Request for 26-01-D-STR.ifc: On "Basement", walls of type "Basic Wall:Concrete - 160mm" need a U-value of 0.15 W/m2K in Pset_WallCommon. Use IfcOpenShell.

First a look at what the model holds.

```python
import ifcopenshell
import ifcopenshell.util.element

model = ifcopenshell.open("26-01-D-STR.ifc")
print(model.schema)
storey = next(s for s in model.by_type("IfcBuildingStorey") if s.Name == "Basement")
walls = [e for e in ifcopenshell.util.element.get_decomposition(storey) if e.is_a("IfcWall")]
seen = {}
for e in walls:
    element_type = ifcopenshell.util.element.get_type(e)
    key = (element_type.Name if element_type != e and element_type else None, ifcopenshell.util.element.get_pset(e, "Pset_WallCommon", "ThermalTransmittance"))
    seen[key] = seen.get(key, 0) + 1
for (name, value), count in sorted(seen.items(), key=str):
    print(count, "x", name, "|", value)
```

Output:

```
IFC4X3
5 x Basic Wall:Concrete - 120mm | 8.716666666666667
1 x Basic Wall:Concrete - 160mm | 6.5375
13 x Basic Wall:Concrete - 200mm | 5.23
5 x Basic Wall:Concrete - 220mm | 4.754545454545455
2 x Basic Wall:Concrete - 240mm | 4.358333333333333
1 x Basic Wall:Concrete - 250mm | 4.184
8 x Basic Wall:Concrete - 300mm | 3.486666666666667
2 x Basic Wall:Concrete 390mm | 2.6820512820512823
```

```python
import ifcopenshell
import ifcopenshell.api.pset
import ifcopenshell.util.element

model = ifcopenshell.open("26-01-D-STR.ifc")

storey = next(s for s in model.by_type("IfcBuildingStorey") if s.Name == "Basement")
walls = [e for e in ifcopenshell.util.element.get_decomposition(storey) if e.is_a("IfcWall")]

count = 0
for e in walls:
    element_type = ifcopenshell.util.element.get_type(e)
    if element_type in (None, e) or element_type.Name != "Basic Wall:Concrete - 160mm":
        continue
    # add_pset returns the element's existing set when there is one.
    pset = ifcopenshell.api.pset.add_pset(model, product=e, name="Pset_WallCommon")
    ifcopenshell.api.pset.edit_pset(model, pset=pset, properties={"ThermalTransmittance": 0.15})
    count += 1

print(count, "walls updated")

model.write("26-01-D-STR_edited.ifc")
```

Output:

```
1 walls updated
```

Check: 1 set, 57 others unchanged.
